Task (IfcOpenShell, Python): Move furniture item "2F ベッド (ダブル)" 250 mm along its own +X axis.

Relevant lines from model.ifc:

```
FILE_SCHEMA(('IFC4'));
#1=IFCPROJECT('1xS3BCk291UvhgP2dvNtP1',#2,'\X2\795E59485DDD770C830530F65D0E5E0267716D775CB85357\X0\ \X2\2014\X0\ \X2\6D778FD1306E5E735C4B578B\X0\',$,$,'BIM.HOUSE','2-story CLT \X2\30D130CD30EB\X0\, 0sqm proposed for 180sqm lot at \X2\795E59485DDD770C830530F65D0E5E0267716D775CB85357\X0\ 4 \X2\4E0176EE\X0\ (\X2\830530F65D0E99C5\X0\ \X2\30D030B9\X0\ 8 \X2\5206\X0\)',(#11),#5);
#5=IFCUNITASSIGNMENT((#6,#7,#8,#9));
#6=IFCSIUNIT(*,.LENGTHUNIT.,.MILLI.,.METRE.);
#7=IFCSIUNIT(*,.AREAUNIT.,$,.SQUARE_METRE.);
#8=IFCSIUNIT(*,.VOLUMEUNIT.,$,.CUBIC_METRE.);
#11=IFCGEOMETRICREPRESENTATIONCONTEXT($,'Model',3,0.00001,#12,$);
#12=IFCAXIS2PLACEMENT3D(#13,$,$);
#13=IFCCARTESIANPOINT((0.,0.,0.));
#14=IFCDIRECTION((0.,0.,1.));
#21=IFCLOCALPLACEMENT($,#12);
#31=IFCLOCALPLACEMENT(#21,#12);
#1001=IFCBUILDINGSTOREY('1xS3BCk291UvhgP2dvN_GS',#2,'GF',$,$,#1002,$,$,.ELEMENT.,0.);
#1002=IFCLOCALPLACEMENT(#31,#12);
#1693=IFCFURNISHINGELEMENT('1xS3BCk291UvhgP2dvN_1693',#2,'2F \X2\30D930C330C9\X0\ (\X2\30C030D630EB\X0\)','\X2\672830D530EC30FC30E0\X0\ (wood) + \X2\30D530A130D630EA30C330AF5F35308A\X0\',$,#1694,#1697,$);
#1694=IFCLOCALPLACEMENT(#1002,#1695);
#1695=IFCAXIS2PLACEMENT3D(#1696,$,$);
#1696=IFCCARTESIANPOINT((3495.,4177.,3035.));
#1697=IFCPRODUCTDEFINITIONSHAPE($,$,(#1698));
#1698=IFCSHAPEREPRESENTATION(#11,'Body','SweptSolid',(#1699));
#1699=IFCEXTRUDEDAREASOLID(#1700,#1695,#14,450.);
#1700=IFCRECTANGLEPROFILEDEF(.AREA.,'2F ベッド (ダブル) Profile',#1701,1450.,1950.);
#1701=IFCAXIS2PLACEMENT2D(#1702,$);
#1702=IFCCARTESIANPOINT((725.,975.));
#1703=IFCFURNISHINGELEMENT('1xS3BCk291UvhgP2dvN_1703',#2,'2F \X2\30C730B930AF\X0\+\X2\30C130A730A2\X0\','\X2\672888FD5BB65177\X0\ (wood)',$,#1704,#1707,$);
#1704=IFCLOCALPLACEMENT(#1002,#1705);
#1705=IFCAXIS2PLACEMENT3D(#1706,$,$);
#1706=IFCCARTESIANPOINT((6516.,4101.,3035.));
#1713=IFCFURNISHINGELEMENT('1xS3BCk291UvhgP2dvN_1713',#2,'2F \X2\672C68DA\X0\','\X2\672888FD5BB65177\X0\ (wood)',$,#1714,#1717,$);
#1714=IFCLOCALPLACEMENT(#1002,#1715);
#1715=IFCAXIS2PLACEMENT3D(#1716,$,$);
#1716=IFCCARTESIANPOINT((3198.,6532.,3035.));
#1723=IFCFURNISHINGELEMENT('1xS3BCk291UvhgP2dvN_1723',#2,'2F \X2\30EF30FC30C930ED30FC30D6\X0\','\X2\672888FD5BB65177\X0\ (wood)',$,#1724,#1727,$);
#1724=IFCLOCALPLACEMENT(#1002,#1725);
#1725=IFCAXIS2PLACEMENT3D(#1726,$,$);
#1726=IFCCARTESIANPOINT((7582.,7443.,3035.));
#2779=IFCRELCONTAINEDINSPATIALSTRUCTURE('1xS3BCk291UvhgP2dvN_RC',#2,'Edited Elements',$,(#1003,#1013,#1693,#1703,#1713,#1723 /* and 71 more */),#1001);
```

```python
import ifcopenshell
import ifcopenshell.api.geometry
import ifcopenshell.util.placement
import ifcopenshell.util.unit

model = ifcopenshell.open("model.ifc")
unit_scale = ifcopenshell.util.unit.calculate_unit_scale(model)

item = model.by_id(1693)
matrix = ifcopenshell.util.placement.get_local_placement(item.ObjectPlacement)
matrix[:3, 3] += matrix[:3, 0] * 0.25 / unit_scale
ifcopenshell.api.geometry.edit_object_placement(model, product=item, matrix=matrix, is_si=False)

print(ifcopenshell.util.placement.get_local_placement(item.ObjectPlacement).round(3) + 0.0)

model.write("model_rev.ifc")
```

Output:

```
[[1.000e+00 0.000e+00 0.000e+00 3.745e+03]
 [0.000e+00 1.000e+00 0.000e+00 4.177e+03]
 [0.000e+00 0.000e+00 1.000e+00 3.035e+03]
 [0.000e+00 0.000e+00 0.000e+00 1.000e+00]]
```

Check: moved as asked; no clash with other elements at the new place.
